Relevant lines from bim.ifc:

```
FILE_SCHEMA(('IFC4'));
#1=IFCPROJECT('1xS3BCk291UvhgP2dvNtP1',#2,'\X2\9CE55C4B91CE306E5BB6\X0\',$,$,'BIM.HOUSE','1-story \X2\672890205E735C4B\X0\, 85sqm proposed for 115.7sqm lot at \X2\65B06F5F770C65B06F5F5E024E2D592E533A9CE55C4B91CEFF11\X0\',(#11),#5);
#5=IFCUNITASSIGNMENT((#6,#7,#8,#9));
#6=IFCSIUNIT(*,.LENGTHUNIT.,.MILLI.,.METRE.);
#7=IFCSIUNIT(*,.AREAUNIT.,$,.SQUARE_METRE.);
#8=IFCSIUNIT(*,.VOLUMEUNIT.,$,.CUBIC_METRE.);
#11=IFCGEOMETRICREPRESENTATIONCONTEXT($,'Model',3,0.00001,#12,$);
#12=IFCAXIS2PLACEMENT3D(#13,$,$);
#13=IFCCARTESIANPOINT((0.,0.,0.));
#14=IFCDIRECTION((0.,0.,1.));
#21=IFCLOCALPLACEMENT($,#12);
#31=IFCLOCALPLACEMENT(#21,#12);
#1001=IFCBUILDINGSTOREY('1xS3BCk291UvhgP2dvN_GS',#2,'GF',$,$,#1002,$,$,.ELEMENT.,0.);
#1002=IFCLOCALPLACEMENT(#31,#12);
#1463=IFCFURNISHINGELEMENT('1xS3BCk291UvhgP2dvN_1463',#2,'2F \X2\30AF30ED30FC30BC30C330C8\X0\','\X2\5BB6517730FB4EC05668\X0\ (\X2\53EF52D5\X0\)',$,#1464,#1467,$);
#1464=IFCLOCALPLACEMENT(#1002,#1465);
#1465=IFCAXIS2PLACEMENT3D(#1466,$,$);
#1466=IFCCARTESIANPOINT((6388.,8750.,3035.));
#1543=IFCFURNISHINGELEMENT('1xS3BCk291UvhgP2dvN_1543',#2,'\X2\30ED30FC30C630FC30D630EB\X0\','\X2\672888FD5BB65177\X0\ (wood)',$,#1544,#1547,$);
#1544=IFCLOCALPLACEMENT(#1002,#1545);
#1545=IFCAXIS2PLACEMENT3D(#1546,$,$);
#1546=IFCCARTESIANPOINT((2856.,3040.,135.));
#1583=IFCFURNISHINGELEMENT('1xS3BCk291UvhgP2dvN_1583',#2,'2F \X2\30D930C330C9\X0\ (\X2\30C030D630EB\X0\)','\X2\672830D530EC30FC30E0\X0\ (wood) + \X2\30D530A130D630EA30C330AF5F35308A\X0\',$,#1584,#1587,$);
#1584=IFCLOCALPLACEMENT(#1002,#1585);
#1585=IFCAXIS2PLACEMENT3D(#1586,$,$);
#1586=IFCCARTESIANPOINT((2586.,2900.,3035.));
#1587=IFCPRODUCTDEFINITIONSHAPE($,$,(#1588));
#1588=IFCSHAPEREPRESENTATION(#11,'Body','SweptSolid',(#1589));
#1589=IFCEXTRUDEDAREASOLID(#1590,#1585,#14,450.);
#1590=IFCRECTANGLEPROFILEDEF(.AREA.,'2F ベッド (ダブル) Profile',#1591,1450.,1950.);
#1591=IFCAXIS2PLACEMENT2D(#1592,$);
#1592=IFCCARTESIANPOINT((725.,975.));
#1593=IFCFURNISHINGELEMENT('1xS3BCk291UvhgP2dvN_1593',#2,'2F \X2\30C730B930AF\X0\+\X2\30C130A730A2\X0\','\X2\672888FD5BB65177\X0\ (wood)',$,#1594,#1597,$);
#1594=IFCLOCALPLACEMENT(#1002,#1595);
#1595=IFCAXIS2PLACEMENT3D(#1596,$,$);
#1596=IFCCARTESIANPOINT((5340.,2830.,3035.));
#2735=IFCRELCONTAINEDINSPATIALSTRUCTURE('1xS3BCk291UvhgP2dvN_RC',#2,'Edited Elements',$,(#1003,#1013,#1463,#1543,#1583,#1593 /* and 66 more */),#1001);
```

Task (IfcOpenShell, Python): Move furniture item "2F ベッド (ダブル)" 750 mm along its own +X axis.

```python
import ifcopenshell
import ifcopenshell.api.geometry
import ifcopenshell.util.placement
import ifcopenshell.util.unit

model = ifcopenshell.open("bim.ifc")
unit_scale = ifcopenshell.util.unit.calculate_unit_scale(model)

item = model.by_guid("1xS3BCk291UvhgP2dvN_1583")
matrix = ifcopenshell.util.placement.get_local_placement(item.ObjectPlacement)
matrix[:3, 3] += matrix[:3, 0] * 0.75 / unit_scale
ifcopenshell.api.geometry.edit_object_placement(model, product=item, matrix=matrix, is_si=False)

print(ifcopenshell.util.placement.get_local_placement(item.ObjectPlacement).round(3) + 0.0)

model.write("bim_v2.ifc")
```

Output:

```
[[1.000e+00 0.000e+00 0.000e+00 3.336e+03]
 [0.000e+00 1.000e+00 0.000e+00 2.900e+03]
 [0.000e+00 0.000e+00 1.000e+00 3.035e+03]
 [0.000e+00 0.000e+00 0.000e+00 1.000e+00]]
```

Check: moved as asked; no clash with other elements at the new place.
